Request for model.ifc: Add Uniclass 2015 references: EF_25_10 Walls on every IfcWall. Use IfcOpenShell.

First a look at what the model holds.

```python
import ifcopenshell

model = ifcopenshell.open("model.ifc")
print(model.schema)
print("classifications:", [c.Name for c in model.by_type("IfcClassification")])
for ifc_class in ("IfcDoor", "IfcRoof", "IfcStair", "IfcWall", "IfcWindow"):
    print(ifc_class, len(model.by_type(ifc_class)))
```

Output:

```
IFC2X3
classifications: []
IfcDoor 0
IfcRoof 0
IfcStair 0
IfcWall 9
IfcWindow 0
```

```python
import ifcopenshell
import ifcopenshell.api.classification

model = ifcopenshell.open("model.ifc")

# IFC2X3 requires Source and Edition and has no link from the project to the system.
system = model.create_entity("IfcClassification", Source="NBS", Edition="2015", Name="Uniclass 2015")

codes = {
    "IfcWall": ("EF_25_10", "Walls"),
}
for ifc_class, (code, name) in codes.items():
    products = model.by_type(ifc_class)
    ifcopenshell.api.classification.add_reference(
        model, products=products, classification=system, identification=code, name=name
    )
    print(code, len(products))

model.write("model_edited.ifc")
```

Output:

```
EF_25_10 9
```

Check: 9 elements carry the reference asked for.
